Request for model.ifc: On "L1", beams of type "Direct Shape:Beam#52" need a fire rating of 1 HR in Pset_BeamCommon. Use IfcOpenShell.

First a look at what the model holds.

```python
import ifcopenshell
import ifcopenshell.util.element

model = ifcopenshell.open("model.ifc")
print(model.schema)
storey = next(s for s in model.by_type("IfcBuildingStorey") if s.Name == "L1")
beams = [e for e in ifcopenshell.util.element.get_decomposition(storey) if e.is_a("IfcBeam")]
seen = {}
for e in beams:
    element_type = ifcopenshell.util.element.get_type(e)
    key = (element_type.Name if element_type != e and element_type else None, ifcopenshell.util.element.get_pset(e, "Pset_BeamCommon", "FireRating"))
    seen[key] = seen.get(key, 0) + 1
for (name, value), count in sorted(seen.items(), key=str):
    print(count, "x", name, "|", value)
```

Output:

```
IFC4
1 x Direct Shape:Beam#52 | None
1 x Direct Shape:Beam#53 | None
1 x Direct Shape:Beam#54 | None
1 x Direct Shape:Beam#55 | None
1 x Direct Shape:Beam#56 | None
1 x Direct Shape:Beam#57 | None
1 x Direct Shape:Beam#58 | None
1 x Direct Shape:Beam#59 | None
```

```python
import ifcopenshell
import ifcopenshell.api.pset
import ifcopenshell.util.element

model = ifcopenshell.open("model.ifc")

storey = next(s for s in model.by_type("IfcBuildingStorey") if s.Name == "L1")
beams = [e for e in ifcopenshell.util.element.get_decomposition(storey) if e.is_a("IfcBeam")]

count = 0
for e in beams:
    element_type = ifcopenshell.util.element.get_type(e)
    if element_type in (None, e) or element_type.Name != "Direct Shape:Beam#52":
        continue
    # add_pset returns the element's existing set when there is one.
    pset = ifcopenshell.api.pset.add_pset(model, product=e, name="Pset_BeamCommon")
    ifcopenshell.api.pset.edit_pset(model, pset=pset, properties={"FireRating": "1 HR"})
    count += 1

print(count, "beams updated")

model.write("model_v2.ifc")
```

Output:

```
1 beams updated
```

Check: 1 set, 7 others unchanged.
